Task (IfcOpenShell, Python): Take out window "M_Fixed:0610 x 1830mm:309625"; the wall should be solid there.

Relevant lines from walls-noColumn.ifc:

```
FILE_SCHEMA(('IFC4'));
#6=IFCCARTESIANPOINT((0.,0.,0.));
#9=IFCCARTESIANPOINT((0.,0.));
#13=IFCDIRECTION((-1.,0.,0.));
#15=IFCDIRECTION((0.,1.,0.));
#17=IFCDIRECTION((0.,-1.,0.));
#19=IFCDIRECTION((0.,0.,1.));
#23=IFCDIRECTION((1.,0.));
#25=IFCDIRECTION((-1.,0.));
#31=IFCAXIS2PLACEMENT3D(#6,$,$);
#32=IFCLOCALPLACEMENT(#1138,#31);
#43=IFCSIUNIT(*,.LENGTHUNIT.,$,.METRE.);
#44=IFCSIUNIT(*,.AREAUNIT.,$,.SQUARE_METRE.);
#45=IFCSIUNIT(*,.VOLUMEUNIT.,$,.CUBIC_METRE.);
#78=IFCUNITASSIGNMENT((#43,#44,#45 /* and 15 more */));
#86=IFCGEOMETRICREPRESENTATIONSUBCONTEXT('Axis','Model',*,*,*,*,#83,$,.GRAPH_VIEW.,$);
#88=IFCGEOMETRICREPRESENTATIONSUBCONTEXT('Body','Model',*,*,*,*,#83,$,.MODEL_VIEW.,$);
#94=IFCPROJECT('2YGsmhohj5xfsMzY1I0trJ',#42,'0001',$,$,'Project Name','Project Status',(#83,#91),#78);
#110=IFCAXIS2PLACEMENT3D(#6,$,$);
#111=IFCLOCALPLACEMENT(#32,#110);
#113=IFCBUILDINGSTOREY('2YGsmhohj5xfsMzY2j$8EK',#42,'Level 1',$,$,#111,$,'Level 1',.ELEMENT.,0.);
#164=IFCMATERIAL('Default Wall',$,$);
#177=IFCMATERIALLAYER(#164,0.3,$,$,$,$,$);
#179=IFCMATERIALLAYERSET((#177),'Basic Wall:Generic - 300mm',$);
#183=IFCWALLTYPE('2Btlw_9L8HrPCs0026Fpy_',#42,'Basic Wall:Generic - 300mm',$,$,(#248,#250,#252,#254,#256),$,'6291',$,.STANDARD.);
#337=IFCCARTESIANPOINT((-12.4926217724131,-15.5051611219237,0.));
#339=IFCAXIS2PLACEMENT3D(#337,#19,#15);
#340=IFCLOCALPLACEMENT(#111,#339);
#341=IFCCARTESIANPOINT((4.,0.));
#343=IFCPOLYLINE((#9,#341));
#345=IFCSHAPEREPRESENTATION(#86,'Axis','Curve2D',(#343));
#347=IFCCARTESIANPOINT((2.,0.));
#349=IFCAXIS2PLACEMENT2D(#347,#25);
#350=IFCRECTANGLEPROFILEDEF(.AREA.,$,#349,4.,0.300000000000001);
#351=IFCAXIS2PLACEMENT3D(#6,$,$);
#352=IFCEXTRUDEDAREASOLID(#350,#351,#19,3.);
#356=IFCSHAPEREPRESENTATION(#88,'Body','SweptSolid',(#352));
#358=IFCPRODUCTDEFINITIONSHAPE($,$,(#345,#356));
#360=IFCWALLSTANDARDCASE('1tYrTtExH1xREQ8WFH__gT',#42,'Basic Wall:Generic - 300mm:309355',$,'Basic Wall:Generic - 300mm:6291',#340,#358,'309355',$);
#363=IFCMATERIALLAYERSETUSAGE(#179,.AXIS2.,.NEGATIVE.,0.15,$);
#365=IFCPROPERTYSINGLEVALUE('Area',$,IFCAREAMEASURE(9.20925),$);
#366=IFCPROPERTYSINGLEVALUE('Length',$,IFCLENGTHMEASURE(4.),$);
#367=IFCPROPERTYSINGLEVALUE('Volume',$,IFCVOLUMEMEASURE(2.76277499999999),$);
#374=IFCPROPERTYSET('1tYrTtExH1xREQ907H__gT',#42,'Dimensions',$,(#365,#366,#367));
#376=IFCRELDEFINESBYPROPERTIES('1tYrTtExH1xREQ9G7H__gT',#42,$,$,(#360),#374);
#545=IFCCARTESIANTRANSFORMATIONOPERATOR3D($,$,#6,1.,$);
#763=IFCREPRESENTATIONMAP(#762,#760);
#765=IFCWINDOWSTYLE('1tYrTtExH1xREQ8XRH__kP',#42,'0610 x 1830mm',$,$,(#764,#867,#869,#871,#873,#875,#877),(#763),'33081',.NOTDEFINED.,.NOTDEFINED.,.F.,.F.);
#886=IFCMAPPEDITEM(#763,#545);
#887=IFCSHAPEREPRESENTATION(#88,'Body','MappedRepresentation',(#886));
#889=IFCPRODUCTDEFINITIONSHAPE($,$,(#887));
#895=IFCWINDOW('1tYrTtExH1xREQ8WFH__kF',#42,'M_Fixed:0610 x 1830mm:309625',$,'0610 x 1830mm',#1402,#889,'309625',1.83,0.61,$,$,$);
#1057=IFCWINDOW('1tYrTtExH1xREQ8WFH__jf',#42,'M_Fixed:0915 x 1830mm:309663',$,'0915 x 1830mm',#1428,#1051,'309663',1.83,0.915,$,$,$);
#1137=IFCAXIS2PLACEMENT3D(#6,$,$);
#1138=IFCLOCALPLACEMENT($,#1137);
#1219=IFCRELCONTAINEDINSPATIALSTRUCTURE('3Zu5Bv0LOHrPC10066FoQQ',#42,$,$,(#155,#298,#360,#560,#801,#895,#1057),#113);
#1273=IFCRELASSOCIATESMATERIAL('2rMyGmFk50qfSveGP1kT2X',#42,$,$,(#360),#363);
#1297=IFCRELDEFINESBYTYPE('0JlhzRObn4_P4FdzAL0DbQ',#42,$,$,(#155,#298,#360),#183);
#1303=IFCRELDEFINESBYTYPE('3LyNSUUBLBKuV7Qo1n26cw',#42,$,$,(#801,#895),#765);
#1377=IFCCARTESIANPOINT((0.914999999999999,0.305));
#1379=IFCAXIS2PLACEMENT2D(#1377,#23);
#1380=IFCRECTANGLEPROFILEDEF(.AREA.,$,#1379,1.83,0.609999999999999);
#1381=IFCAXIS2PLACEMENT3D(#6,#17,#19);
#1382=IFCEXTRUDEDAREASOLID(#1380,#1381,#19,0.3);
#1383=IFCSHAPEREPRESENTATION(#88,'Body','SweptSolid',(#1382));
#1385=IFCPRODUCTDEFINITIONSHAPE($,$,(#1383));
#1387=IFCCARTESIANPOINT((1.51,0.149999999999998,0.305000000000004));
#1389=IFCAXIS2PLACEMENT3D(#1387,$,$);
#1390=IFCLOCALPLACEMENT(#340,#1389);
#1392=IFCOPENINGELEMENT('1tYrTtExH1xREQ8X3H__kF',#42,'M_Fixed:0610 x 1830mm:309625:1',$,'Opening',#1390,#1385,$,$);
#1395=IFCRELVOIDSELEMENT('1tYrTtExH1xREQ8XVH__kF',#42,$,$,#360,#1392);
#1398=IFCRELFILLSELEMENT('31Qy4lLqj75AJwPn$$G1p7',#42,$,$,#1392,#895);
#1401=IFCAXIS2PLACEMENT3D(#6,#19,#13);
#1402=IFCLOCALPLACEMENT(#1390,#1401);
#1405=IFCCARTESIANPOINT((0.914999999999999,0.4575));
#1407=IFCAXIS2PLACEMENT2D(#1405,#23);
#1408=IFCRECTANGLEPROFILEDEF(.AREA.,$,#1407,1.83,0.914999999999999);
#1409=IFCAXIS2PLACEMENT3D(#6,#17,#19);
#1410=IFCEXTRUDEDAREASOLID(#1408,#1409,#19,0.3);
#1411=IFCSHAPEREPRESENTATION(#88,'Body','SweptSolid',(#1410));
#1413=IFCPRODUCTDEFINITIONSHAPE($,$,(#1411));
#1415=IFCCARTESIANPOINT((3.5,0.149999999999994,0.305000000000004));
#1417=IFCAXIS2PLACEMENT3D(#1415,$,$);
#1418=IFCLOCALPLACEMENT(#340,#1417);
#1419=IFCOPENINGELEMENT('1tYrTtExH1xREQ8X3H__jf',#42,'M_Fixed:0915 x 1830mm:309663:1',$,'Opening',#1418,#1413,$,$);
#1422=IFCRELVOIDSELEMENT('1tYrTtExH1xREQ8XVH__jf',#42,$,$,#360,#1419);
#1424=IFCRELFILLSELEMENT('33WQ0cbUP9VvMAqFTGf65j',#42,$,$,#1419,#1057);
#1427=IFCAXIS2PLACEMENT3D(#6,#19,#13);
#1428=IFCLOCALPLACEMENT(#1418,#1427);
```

```python
import ifcopenshell
import ifcopenshell.api.feature
import ifcopenshell.api.pset
import ifcopenshell.api.root
import ifcopenshell.geom
import ifcopenshell.util.element
import ifcopenshell.util.shape
import ifcopenshell.util.unit

model = ifcopenshell.open("walls-noColumn.ifc")
area_scale = ifcopenshell.util.unit.calculate_unit_scale(model, "AREAUNIT")
volume_scale = ifcopenshell.util.unit.calculate_unit_scale(model, "VOLUMEUNIT")
settings = ifcopenshell.geom.settings()


def volume(element):
    """Net volume in cubic metres, openings subtracted."""
    shape = ifcopenshell.geom.create_shape(settings, element)
    return ifcopenshell.util.shape.get_volume(shape.geometry)


window = model.by_guid("1tYrTtExH1xREQ8WFH__kF")
opening = window.FillsVoids[0].RelatingOpeningElement
wall = opening.VoidsElements[0].RelatingBuildingElement
before = volume(wall)

ifcopenshell.api.root.remove_product(model, product=window)
ifcopenshell.api.feature.remove_feature(model, feature=opening)

after = volume(wall)
thickness = 0.3  # wall thickness in metres

# Update the wall's stored quantities.
pset = model.by_id(ifcopenshell.util.element.get_pset(wall, "Dimensions", should_inherit=False)["id"])
ifcopenshell.api.pset.edit_pset(model, pset=pset, properties={
    "Area": model.create_entity("IfcAreaMeasure", after / thickness / area_scale),
    "Volume": model.create_entity("IfcVolumeMeasure", after / volume_scale),
})

print(f"wall volume {before:.3f} -> {after:.3f} m3")

model.write("walls-noColumn_updated.ifc")
```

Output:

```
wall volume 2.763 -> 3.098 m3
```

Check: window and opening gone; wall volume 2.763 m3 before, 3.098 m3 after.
